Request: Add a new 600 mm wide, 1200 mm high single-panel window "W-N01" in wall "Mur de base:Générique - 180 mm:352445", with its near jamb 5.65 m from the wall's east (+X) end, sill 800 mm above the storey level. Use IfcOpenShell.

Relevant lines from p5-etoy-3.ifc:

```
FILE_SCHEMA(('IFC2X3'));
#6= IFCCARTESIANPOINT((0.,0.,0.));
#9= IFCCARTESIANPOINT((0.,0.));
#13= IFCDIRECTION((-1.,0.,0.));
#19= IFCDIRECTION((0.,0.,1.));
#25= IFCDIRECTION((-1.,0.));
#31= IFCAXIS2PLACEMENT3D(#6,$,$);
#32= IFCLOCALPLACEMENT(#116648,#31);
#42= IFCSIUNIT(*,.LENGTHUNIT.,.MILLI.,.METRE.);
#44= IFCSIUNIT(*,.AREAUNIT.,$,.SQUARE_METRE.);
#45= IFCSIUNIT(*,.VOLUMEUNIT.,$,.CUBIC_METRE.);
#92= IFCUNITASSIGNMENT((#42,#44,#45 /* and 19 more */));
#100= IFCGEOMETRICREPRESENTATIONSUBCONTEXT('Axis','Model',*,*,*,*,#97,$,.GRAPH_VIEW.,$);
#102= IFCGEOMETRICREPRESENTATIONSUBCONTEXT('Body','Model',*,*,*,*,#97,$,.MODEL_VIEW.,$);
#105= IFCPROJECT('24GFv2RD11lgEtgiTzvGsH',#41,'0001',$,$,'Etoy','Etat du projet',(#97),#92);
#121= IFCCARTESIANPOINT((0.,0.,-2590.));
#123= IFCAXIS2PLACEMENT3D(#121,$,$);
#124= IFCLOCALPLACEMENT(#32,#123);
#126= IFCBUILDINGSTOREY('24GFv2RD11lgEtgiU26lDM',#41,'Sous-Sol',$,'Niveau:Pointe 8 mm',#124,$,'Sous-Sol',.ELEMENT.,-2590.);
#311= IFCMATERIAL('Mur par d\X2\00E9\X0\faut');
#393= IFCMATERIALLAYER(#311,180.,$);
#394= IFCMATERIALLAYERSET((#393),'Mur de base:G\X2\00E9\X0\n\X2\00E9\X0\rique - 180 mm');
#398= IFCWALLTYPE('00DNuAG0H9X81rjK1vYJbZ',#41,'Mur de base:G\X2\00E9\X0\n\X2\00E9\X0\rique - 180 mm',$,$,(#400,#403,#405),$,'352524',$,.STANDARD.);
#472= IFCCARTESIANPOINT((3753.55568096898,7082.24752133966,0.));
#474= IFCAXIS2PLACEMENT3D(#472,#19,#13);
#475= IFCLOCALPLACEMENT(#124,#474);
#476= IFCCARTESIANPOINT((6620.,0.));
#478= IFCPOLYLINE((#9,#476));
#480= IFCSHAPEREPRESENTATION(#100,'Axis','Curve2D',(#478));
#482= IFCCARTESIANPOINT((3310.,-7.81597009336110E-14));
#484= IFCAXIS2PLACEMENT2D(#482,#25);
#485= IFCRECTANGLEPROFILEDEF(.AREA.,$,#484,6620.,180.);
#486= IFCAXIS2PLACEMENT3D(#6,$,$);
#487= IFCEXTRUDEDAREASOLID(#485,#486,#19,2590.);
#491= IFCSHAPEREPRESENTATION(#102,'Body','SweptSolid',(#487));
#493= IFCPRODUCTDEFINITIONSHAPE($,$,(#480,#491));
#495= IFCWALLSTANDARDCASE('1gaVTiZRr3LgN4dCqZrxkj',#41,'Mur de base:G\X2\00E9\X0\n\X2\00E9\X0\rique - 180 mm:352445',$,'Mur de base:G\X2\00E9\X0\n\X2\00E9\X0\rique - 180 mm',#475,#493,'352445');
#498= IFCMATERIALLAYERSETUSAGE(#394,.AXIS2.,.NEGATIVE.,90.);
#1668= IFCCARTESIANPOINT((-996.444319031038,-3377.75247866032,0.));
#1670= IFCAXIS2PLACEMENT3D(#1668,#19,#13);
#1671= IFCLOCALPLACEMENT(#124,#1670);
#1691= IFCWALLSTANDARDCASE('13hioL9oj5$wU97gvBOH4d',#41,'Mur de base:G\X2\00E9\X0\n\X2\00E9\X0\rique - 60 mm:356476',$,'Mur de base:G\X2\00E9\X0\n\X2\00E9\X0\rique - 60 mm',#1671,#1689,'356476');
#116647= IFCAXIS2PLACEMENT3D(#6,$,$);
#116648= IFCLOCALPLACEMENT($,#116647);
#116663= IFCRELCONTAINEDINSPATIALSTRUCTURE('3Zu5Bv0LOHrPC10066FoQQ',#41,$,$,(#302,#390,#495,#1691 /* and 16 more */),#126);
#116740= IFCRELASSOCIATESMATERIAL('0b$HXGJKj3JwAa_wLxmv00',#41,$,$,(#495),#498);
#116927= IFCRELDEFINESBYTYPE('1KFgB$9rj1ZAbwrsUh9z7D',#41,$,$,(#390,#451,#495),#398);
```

```python
import numpy as np
import ifcopenshell
import ifcopenshell.api.feature
import ifcopenshell.api.geometry
import ifcopenshell.api.root
import ifcopenshell.api.spatial
import ifcopenshell.api.type
import ifcopenshell.geom
import ifcopenshell.util.element
import ifcopenshell.util.placement
import ifcopenshell.util.representation
import ifcopenshell.util.shape
import ifcopenshell.util.unit

model = ifcopenshell.open("p5-etoy-3.ifc")
unit_scale = ifcopenshell.util.unit.calculate_unit_scale(model)
settings = ifcopenshell.geom.settings()


def volume(element):
    """Net volume in cubic metres, openings subtracted."""
    shape = ifcopenshell.geom.create_shape(settings, element)
    return ifcopenshell.util.shape.get_volume(shape.geometry)


wall = model.by_id(495)
storey = ifcopenshell.util.element.get_container(wall, ifc_class="IfcBuildingStorey")
context = ifcopenshell.util.representation.get_context(model, "Model", "Body", "MODEL_VIEW")
before = volume(wall)

width, height, from_end, sill = 0.6, 1.2, 5.65, 0.8  # metres

# The wall runs along its own X axis, and the end named is its -X end.
wall_shape = ifcopenshell.geom.create_shape(settings, wall)
x, y, z = ifcopenshell.util.shape.get_vertices(wall_shape.geometry).T
start = x.min() + from_end
face, thickness = float(y.min()), float(y.max() - y.min())
wall_matrix = ifcopenshell.util.placement.get_local_placement(wall.ObjectPlacement)
level = ifcopenshell.util.placement.get_local_placement(storey.ObjectPlacement)[2, 3]


def in_wall(x, y):
    """Placement at x, y metres in the wall's axes, at sill height."""
    matrix = wall_matrix.copy()
    matrix[:, 3] = wall_matrix @ np.array([x / unit_scale, y / unit_scale, 0.0, 1.0])
    matrix[2, 3] = level + sill / unit_scale
    return matrix


# Opening: a box that overshoots both wall faces by 50 mm.
opening = ifcopenshell.api.root.create_entity(model, ifc_class="IfcOpeningElement")
box = ifcopenshell.api.geometry.add_wall_representation(
    model, context=context, length=width, height=height, thickness=thickness + 0.1
)
ifcopenshell.api.geometry.assign_representation(model, product=opening, representation=box)
ifcopenshell.api.geometry.edit_object_placement(model, product=opening, matrix=in_wall(start, face - 0.05), is_si=False)
ifcopenshell.api.feature.add_feature(model, feature=opening, element=wall)

window = ifcopenshell.api.root.create_entity(model, ifc_class="IfcWindow", name="W-N01")
window.OverallWidth, window.OverallHeight = width / unit_scale, height / unit_scale
body = ifcopenshell.api.geometry.add_window_representation(
    model,
    context=context,
    overall_width=window.OverallWidth,
    overall_height=window.OverallHeight,
    partition_type="SINGLE_PANEL",
)
ifcopenshell.api.geometry.assign_representation(model, product=window, representation=body)
ifcopenshell.api.spatial.assign_container(model, products=[window], relating_structure=storey)
fills = ifcopenshell.api.feature.add_filling(model, opening=opening, element=window)
fills.OwnerHistory = window.OwnerHistory  # required in IFC2X3

# IFC2X3 keeps the operation on the window style.
style = ifcopenshell.api.root.create_entity(model, ifc_class="IfcWindowStyle", name="W-N01")
style.OperationType, style.ConstructionType = "SINGLE_PANEL", "NOTDEFINED"
style.ParameterTakesPrecedence = style.Sizeable = False
ifcopenshell.api.type.assign_type(model, related_objects=[window], relating_type=style)

# Centre the window in the wall's thickness.
ifcopenshell.api.geometry.edit_object_placement(model, product=window, matrix=in_wall(start, face), is_si=False)
window_shape = ifcopenshell.geom.create_shape(settings, window)
depth = ifcopenshell.util.shape.get_vertices(window_shape.geometry)[:, 1]
offset = face + thickness / 2 - (depth.min() + depth.max()) / 2
ifcopenshell.api.geometry.edit_object_placement(model, product=window, matrix=in_wall(start, offset), is_si=False)

after = volume(wall)

print(f"wall volume {before:.3f} -> {after:.3f} m3")

model.write("p5-etoy-3_rev.ifc")
```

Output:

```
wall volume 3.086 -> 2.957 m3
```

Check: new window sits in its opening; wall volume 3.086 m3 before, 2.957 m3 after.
